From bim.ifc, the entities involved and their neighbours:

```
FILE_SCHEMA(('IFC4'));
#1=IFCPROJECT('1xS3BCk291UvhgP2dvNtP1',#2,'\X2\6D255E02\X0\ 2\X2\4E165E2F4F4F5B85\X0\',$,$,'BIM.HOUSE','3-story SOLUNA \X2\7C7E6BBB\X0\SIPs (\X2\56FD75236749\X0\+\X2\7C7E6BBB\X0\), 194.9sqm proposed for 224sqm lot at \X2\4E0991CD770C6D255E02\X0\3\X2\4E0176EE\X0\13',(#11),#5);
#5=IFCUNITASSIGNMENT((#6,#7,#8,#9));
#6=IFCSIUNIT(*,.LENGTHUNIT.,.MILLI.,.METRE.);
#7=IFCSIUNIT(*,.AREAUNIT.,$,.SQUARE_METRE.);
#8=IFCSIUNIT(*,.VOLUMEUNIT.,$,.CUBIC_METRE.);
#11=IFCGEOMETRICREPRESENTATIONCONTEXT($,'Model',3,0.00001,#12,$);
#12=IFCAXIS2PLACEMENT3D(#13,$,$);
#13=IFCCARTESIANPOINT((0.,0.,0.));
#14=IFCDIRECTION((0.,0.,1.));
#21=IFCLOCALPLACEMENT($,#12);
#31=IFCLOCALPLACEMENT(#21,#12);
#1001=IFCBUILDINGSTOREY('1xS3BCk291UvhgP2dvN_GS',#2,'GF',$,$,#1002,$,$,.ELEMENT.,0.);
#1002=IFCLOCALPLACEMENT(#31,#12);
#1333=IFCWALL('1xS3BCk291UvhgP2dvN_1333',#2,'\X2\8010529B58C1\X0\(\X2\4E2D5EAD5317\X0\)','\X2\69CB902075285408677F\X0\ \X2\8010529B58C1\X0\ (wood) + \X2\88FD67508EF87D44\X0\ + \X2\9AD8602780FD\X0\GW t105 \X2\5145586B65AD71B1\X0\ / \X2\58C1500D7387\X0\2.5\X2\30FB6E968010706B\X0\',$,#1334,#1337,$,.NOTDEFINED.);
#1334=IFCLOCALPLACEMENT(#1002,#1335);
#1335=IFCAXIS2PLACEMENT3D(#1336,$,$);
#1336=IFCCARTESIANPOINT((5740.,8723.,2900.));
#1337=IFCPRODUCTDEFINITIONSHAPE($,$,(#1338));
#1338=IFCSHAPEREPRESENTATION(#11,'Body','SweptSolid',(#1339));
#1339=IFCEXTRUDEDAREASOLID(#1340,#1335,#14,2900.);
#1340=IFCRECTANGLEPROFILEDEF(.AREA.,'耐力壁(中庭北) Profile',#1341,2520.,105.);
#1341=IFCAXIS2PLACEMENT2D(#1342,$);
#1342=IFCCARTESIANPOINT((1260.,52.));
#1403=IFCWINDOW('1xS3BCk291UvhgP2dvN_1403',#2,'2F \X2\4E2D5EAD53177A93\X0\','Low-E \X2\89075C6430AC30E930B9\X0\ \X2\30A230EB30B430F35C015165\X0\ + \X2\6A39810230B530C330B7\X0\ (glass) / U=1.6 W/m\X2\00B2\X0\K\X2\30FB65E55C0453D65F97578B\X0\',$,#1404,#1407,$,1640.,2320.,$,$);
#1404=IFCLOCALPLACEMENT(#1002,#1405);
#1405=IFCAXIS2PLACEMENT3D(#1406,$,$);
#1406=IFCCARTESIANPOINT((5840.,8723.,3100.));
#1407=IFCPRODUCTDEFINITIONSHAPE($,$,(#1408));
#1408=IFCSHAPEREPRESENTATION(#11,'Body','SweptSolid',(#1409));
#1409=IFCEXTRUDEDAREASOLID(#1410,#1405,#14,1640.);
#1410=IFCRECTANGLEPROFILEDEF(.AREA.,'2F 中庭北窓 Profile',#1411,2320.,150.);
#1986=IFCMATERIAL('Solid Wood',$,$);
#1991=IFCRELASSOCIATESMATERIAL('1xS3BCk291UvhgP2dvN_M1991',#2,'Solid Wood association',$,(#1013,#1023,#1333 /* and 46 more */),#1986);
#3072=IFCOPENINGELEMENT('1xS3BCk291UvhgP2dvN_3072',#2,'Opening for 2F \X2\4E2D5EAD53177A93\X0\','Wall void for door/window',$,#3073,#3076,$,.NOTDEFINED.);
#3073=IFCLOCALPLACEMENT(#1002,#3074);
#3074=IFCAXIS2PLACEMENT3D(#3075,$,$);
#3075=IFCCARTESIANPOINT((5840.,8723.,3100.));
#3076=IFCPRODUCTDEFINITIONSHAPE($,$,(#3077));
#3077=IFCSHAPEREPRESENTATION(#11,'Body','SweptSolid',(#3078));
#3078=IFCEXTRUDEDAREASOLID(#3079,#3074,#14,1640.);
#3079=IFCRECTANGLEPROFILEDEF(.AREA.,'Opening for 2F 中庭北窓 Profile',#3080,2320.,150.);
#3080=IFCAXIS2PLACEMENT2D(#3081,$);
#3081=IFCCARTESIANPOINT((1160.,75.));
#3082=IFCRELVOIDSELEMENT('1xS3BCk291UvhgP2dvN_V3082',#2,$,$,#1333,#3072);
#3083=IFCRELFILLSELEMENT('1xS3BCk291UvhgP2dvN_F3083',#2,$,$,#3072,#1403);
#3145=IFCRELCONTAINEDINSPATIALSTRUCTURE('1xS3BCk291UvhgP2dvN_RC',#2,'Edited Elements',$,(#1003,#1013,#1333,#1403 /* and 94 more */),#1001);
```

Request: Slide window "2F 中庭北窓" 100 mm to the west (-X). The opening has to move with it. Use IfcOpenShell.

```python
import ifcopenshell
import ifcopenshell.api.geometry
import ifcopenshell.util.placement

model = ifcopenshell.open("bim.ifc")

window = model.by_guid("1xS3BCk291UvhgP2dvN_1403")
opening = window.FillsVoids[0].RelatingOpeningElement
wall = opening.VoidsElements[0].RelatingBuildingElement

wall_matrix = ifcopenshell.util.placement.get_local_placement(wall.ObjectPlacement)
shift = wall_matrix[:3, 0] * -100.0
before = ifcopenshell.util.placement.get_local_placement(window.ObjectPlacement)[:3, 3].copy()

# The window is not placed relative to its opening, so move both.
for product in (opening, window):
    matrix = ifcopenshell.util.placement.get_local_placement(product.ObjectPlacement)
    matrix[:3, 3] += shift
    ifcopenshell.api.geometry.edit_object_placement(model, product=product, matrix=matrix, is_si=False)

after = ifcopenshell.util.placement.get_local_placement(window.ObjectPlacement)[:3, 3]
print("window moved by", (after - before).round(3) + 0.0)

model.write("bim_v2.ifc")
```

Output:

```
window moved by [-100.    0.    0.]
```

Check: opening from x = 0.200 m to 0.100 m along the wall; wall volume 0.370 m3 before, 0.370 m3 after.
